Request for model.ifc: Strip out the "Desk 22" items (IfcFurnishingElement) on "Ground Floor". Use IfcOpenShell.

First a look at what the model holds.

```python
import ifcopenshell
import ifcopenshell.util.element

model = ifcopenshell.open("model.ifc")
print(model.schema)
storey = next(s for s in model.by_type("IfcBuildingStorey") if s.Name == "Ground Floor")
furniture = [e for e in ifcopenshell.util.element.get_decomposition(storey) if e.is_a("IfcFurnishingElement")]
seen = {}
for e in furniture:
    element_type = ifcopenshell.util.element.get_type(e)
    name = element_type.Name if element_type not in (None, e) else None
    seen[name] = seen.get(name, 0) + 1
for name, count in sorted(seen.items(), key=str):
    print(count, "x", name)
```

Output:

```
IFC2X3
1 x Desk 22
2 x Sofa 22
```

```python
import ifcopenshell
import ifcopenshell.api.root
import ifcopenshell.util.element

model = ifcopenshell.open("model.ifc")

storey = next(s for s in model.by_type("IfcBuildingStorey") if s.Name == "Ground Floor")
furniture = [e for e in ifcopenshell.util.element.get_decomposition(storey) if e.is_a("IfcFurnishingElement")]
targets = [e for e in furniture if (t := ifcopenshell.util.element.get_type(e)) not in (None, e) and t.Name == "Desk 22"]

for e in targets:
    ifcopenshell.api.root.remove_product(model, product=e)
print(len(targets), "removed")

model.write("model_edited.ifc")
```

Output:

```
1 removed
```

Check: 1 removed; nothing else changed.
